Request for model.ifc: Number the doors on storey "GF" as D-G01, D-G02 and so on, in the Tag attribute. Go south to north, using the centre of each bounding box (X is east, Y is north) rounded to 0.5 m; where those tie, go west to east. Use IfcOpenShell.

First a look at what the model holds.

```python
import ifcopenshell
import ifcopenshell.util.element
import ifcopenshell.util.placement

model = ifcopenshell.open("model.ifc")
print(model.schema)
storey = next(s for s in model.by_type("IfcBuildingStorey") if s.Name == "GF")
doors = [e for e in ifcopenshell.util.element.get_decomposition(storey) if e.is_a("IfcDoor")]
for e in sorted(doors, key=lambda e: e.id()):
    origin = ifcopenshell.util.placement.get_local_placement(e.ObjectPlacement)[:3, 3]
    print(e.id(), e.Tag, e.Name, origin.round(2) + 0.0, sep=" | ")
```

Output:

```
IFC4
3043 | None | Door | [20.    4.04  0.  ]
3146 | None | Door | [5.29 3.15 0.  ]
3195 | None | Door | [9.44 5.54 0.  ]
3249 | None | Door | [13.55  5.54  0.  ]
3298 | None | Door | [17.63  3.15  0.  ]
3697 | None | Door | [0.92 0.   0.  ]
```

```python
import ifcopenshell
import ifcopenshell.geom
import ifcopenshell.util.element
import ifcopenshell.util.shape

model = ifcopenshell.open("model.ifc")
settings = ifcopenshell.geom.settings()
settings.set("use-world-coords", True)


def centre(element):
    shape = ifcopenshell.geom.create_shape(settings, element)
    return ifcopenshell.util.shape.get_bbox_centroid(shape.geometry)


storey = next(s for s in model.by_type("IfcBuildingStorey") if s.Name == "GF")
doors = [e for e in ifcopenshell.util.element.get_decomposition(storey) if e.is_a("IfcDoor")]

# Insertion points can sit at a corner or the storey origin, so sort by the geometry (in metres).
centres = {e: centre(e) for e in doors}
doors.sort(key=lambda e: (round(centres[e][1] / 0.5), centres[e][0]))

for i, e in enumerate(doors, start=1):
    number = f"D-G{i:02d}"
    e.Tag = number
    print(e.id(), number)

model.write("model-out.ifc")
```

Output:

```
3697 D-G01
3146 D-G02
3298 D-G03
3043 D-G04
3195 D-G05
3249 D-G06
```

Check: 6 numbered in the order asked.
